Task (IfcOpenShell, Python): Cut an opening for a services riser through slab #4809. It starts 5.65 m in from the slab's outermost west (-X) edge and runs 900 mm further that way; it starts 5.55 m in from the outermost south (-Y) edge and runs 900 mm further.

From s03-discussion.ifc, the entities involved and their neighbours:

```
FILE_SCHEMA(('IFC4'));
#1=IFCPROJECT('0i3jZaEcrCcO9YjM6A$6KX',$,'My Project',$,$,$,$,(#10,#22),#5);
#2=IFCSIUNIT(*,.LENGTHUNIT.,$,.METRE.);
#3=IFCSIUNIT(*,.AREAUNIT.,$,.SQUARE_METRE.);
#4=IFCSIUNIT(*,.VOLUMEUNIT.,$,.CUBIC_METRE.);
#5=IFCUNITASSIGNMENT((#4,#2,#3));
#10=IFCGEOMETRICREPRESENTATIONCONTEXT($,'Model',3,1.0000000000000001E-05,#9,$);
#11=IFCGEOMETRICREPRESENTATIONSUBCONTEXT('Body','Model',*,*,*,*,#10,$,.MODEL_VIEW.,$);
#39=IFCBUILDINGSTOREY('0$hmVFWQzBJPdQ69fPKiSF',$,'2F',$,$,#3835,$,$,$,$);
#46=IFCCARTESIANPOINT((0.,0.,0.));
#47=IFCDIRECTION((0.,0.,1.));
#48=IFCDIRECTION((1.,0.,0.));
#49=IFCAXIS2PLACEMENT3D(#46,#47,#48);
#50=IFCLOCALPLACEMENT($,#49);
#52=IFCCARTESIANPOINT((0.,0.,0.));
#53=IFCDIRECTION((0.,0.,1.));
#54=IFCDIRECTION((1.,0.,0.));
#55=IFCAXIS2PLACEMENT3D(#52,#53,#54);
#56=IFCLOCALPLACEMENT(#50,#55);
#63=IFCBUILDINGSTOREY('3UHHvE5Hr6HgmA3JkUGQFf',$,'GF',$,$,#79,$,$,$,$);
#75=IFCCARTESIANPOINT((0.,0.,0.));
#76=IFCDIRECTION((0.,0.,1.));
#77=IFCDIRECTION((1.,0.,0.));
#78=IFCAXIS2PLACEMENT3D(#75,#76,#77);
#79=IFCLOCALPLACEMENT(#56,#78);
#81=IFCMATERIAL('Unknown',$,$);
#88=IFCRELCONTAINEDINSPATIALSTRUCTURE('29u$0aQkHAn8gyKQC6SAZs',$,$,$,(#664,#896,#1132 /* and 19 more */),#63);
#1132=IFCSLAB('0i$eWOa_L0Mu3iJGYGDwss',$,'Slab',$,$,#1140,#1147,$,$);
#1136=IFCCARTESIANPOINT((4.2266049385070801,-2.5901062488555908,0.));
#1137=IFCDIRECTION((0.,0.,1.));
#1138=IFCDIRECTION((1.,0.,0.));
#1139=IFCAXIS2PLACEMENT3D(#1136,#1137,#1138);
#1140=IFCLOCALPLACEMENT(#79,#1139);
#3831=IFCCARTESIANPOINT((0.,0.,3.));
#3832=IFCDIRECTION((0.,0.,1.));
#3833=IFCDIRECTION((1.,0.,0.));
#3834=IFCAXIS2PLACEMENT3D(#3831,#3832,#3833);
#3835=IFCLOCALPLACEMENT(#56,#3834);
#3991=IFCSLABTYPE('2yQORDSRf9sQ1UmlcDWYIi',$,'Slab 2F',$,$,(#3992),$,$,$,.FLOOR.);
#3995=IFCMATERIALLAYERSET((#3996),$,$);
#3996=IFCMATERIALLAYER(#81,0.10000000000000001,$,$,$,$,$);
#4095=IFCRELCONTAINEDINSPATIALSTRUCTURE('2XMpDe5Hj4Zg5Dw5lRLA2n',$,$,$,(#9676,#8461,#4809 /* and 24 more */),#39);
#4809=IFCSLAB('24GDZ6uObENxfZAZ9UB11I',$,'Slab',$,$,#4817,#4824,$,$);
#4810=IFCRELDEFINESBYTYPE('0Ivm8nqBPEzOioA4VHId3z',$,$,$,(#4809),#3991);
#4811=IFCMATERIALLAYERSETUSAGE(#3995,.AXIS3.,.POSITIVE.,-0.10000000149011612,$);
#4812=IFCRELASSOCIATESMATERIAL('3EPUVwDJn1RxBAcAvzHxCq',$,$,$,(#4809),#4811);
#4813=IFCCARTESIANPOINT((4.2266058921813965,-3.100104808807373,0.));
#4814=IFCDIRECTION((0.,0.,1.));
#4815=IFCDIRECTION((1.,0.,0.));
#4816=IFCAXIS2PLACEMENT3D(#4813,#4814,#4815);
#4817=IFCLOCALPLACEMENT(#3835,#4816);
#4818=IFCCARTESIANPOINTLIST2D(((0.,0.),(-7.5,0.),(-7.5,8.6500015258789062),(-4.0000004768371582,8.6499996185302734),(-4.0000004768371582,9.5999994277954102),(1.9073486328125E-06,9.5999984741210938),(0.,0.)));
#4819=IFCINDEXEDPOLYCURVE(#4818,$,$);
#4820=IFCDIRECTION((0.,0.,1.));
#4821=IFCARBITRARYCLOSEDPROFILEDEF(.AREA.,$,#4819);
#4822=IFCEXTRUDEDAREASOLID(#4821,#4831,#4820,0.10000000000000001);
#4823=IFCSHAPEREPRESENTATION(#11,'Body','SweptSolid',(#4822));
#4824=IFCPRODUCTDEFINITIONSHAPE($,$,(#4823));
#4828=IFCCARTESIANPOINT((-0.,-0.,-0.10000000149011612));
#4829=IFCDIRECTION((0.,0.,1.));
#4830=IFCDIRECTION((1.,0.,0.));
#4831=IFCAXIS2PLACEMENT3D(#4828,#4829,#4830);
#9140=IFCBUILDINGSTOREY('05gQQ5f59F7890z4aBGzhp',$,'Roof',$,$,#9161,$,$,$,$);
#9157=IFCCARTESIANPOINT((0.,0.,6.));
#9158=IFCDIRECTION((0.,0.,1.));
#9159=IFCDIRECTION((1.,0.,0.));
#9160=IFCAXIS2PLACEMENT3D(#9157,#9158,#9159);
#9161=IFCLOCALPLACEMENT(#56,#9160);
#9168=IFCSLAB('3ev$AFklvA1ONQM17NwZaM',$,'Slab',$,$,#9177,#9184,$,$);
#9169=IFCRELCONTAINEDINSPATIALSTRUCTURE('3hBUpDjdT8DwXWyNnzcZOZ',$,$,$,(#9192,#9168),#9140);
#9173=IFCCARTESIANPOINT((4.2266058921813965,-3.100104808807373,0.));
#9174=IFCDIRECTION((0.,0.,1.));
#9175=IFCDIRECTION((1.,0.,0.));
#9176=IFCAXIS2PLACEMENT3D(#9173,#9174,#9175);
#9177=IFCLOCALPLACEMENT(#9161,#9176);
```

```python
import numpy as np
import ifcopenshell
import ifcopenshell.api.feature
import ifcopenshell.api.geometry
import ifcopenshell.api.root
import ifcopenshell.geom
import ifcopenshell.util.placement
import ifcopenshell.util.representation
import ifcopenshell.util.shape
import ifcopenshell.util.unit

model = ifcopenshell.open("s03-discussion.ifc")
unit_scale = ifcopenshell.util.unit.calculate_unit_scale(model)
settings = ifcopenshell.geom.settings()


def volume(element):
    """Net volume in cubic metres, openings subtracted."""
    shape = ifcopenshell.geom.create_shape(settings, element)
    return ifcopenshell.util.shape.get_volume(shape.geometry)


slab = model.by_guid("24GDZ6uObENxfZAZ9UB11I")
before = volume(slab)

# Extent in the slab's own axes, in metres. The edges named are its -X and -Y sides.
slab_shape = ifcopenshell.geom.create_shape(settings, slab)
vertices = ifcopenshell.util.shape.get_vertices(slab_shape.geometry)
x_min, y_min, bottom = vertices.min(axis=0)
top = vertices[:, 2].max()

opening = ifcopenshell.api.root.create_entity(model, ifc_class="IfcOpeningElement", name="Services riser opening", predefined_type="OPENING")
context = ifcopenshell.util.representation.get_context(model, "Model", "Body", "MODEL_VIEW")
width, depth = 0.9, 0.9
outline = [(0.0, 0.0), (width, 0.0), (width, depth), (0.0, depth), (0.0, 0.0)]
# Overshoot both faces by 50 mm so the cut is clean.
shape = ifcopenshell.api.geometry.add_slab_representation(
    model, context=context, depth=top - bottom + 0.1, polyline=outline
)
ifcopenshell.api.geometry.assign_representation(model, product=opening, representation=shape)

matrix = ifcopenshell.util.placement.get_local_placement(slab.ObjectPlacement)
matrix[:, 3] = matrix @ np.append(np.array([x_min + 5.65, y_min + 5.55, bottom - 0.05]) / unit_scale, 1.0)
ifcopenshell.api.geometry.edit_object_placement(model, product=opening, matrix=matrix, is_si=False)
ifcopenshell.api.feature.add_feature(model, feature=opening, element=slab)

after = volume(slab)

print(f"slab volume {before:.3f} -> {after:.3f} m3")

model.write("s03-discussion_rev.ifc")
```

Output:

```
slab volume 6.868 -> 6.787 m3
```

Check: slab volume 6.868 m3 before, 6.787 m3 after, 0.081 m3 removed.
